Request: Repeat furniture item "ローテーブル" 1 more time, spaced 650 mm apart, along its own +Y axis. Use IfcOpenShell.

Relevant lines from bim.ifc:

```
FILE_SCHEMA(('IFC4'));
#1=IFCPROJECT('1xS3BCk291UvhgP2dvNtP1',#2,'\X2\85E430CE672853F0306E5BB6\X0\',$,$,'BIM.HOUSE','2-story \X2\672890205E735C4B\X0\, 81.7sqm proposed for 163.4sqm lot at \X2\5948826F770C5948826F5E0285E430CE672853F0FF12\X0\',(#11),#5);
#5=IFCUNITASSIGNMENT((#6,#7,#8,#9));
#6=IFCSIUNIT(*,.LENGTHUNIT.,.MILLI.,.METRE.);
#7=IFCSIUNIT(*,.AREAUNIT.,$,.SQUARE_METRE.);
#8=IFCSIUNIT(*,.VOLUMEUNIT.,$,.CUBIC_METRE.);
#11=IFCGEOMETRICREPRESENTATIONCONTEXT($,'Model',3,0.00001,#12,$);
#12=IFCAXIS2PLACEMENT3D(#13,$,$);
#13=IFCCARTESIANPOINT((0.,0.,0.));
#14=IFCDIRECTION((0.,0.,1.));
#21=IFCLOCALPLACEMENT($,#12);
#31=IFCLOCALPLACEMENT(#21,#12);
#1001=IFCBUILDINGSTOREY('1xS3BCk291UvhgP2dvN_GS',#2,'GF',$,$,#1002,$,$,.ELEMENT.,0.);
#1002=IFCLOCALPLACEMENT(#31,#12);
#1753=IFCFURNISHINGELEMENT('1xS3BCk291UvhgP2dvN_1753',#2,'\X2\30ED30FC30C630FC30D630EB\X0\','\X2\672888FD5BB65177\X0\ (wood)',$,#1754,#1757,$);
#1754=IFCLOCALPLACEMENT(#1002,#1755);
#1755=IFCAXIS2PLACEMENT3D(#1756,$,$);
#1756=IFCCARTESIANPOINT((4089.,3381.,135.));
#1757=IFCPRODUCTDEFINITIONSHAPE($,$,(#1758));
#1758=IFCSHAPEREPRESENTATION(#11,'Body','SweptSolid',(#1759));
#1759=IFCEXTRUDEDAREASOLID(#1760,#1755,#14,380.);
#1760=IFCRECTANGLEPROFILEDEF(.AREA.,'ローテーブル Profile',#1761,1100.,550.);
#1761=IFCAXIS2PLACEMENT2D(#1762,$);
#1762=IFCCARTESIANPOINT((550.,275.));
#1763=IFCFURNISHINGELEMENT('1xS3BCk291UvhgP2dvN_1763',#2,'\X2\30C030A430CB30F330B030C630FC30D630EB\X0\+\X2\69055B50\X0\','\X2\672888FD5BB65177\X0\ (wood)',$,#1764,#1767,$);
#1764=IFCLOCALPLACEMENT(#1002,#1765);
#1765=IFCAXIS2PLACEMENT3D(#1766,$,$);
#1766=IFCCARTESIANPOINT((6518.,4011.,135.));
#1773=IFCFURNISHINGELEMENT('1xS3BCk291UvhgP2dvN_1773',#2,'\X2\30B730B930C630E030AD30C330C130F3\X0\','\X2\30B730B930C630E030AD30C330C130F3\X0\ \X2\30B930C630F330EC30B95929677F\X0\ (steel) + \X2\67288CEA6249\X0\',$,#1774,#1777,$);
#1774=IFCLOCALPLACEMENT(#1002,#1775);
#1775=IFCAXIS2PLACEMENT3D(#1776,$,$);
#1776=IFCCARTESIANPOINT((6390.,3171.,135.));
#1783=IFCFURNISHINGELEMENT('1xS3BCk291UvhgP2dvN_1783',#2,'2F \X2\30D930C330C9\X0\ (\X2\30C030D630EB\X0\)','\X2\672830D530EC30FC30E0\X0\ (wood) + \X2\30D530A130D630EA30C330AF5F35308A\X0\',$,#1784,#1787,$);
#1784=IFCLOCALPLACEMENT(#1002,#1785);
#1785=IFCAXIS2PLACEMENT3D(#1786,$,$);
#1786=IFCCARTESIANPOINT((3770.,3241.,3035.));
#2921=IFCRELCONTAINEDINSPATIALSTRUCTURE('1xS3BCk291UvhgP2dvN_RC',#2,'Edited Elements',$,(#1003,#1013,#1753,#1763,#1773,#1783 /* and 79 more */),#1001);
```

```python
import ifcopenshell
import ifcopenshell.api.geometry
import ifcopenshell.api.root
import ifcopenshell.util.element
import ifcopenshell.util.placement

model = ifcopenshell.open("bim.ifc")


def reuse_history(source, copy):
    """copy_class also copies each property set's owner history, people and application; keep the originals."""
    for rel in copy.IsDefinedBy:
        if rel.is_a("IfcRelDefinesByProperties") and (history := rel.RelatingPropertyDefinition.OwnerHistory):
            rel.RelatingPropertyDefinition.OwnerHistory = source.OwnerHistory
            ifcopenshell.util.element.remove_deep2(model, history)


source = model.by_guid("1xS3BCk291UvhgP2dvN_1753")
base = ifcopenshell.util.placement.get_local_placement(source.ObjectPlacement)
step = base[:3, 1] * 650.0

for i in range(1, 2):
    copy = ifcopenshell.api.root.copy_class(model, product=source)
    copy.Representation = ifcopenshell.util.element.copy_deep(
        model, source.Representation, exclude=["IfcGeometricRepresentationContext", "IfcRepresentationMap"]
    )
    reuse_history(source, copy)
    matrix = base.copy()
    matrix[:3, 3] += i * step
    print("added at", matrix[:3, 3].round(3) + 0.0)
    ifcopenshell.api.geometry.edit_object_placement(model, product=copy, matrix=matrix, is_si=False)

model.write("bim_edited.ifc")
```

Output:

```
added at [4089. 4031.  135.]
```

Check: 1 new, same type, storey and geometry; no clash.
